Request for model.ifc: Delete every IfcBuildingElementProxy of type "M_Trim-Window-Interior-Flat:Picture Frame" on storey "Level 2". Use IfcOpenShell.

First a look at what the model holds.

```python
import ifcopenshell
import ifcopenshell.util.element

model = ifcopenshell.open("model.ifc")
print(model.schema)
storey = next(s for s in model.by_type("IfcBuildingStorey") if s.Name == "Level 2")
proxies = [e for e in ifcopenshell.util.element.get_decomposition(storey) if e.is_a("IfcBuildingElementProxy")]
seen = {}
for e in proxies:
    element_type = ifcopenshell.util.element.get_type(e)
    name = element_type.Name if element_type not in (None, e) else None
    seen[name] = seen.get(name, 0) + 1
for name, count in sorted(seen.items(), key=str):
    print(count, "x", name)
```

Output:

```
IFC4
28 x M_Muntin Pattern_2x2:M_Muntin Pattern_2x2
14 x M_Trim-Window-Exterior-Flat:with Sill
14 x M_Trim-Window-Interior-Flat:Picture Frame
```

```python
import ifcopenshell
import ifcopenshell.api.root
import ifcopenshell.util.element

model = ifcopenshell.open("model.ifc")

storey = next(s for s in model.by_type("IfcBuildingStorey") if s.Name == "Level 2")
proxies = [e for e in ifcopenshell.util.element.get_decomposition(storey) if e.is_a("IfcBuildingElementProxy")]
targets = [e for e in proxies if (t := ifcopenshell.util.element.get_type(e)) not in (None, e) and t.Name == "M_Trim-Window-Interior-Flat:Picture Frame"]

for e in targets:
    ifcopenshell.api.root.remove_product(model, product=e)
print(len(targets), "removed")

model.write("model_edited.ifc")
```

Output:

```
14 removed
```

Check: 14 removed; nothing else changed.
